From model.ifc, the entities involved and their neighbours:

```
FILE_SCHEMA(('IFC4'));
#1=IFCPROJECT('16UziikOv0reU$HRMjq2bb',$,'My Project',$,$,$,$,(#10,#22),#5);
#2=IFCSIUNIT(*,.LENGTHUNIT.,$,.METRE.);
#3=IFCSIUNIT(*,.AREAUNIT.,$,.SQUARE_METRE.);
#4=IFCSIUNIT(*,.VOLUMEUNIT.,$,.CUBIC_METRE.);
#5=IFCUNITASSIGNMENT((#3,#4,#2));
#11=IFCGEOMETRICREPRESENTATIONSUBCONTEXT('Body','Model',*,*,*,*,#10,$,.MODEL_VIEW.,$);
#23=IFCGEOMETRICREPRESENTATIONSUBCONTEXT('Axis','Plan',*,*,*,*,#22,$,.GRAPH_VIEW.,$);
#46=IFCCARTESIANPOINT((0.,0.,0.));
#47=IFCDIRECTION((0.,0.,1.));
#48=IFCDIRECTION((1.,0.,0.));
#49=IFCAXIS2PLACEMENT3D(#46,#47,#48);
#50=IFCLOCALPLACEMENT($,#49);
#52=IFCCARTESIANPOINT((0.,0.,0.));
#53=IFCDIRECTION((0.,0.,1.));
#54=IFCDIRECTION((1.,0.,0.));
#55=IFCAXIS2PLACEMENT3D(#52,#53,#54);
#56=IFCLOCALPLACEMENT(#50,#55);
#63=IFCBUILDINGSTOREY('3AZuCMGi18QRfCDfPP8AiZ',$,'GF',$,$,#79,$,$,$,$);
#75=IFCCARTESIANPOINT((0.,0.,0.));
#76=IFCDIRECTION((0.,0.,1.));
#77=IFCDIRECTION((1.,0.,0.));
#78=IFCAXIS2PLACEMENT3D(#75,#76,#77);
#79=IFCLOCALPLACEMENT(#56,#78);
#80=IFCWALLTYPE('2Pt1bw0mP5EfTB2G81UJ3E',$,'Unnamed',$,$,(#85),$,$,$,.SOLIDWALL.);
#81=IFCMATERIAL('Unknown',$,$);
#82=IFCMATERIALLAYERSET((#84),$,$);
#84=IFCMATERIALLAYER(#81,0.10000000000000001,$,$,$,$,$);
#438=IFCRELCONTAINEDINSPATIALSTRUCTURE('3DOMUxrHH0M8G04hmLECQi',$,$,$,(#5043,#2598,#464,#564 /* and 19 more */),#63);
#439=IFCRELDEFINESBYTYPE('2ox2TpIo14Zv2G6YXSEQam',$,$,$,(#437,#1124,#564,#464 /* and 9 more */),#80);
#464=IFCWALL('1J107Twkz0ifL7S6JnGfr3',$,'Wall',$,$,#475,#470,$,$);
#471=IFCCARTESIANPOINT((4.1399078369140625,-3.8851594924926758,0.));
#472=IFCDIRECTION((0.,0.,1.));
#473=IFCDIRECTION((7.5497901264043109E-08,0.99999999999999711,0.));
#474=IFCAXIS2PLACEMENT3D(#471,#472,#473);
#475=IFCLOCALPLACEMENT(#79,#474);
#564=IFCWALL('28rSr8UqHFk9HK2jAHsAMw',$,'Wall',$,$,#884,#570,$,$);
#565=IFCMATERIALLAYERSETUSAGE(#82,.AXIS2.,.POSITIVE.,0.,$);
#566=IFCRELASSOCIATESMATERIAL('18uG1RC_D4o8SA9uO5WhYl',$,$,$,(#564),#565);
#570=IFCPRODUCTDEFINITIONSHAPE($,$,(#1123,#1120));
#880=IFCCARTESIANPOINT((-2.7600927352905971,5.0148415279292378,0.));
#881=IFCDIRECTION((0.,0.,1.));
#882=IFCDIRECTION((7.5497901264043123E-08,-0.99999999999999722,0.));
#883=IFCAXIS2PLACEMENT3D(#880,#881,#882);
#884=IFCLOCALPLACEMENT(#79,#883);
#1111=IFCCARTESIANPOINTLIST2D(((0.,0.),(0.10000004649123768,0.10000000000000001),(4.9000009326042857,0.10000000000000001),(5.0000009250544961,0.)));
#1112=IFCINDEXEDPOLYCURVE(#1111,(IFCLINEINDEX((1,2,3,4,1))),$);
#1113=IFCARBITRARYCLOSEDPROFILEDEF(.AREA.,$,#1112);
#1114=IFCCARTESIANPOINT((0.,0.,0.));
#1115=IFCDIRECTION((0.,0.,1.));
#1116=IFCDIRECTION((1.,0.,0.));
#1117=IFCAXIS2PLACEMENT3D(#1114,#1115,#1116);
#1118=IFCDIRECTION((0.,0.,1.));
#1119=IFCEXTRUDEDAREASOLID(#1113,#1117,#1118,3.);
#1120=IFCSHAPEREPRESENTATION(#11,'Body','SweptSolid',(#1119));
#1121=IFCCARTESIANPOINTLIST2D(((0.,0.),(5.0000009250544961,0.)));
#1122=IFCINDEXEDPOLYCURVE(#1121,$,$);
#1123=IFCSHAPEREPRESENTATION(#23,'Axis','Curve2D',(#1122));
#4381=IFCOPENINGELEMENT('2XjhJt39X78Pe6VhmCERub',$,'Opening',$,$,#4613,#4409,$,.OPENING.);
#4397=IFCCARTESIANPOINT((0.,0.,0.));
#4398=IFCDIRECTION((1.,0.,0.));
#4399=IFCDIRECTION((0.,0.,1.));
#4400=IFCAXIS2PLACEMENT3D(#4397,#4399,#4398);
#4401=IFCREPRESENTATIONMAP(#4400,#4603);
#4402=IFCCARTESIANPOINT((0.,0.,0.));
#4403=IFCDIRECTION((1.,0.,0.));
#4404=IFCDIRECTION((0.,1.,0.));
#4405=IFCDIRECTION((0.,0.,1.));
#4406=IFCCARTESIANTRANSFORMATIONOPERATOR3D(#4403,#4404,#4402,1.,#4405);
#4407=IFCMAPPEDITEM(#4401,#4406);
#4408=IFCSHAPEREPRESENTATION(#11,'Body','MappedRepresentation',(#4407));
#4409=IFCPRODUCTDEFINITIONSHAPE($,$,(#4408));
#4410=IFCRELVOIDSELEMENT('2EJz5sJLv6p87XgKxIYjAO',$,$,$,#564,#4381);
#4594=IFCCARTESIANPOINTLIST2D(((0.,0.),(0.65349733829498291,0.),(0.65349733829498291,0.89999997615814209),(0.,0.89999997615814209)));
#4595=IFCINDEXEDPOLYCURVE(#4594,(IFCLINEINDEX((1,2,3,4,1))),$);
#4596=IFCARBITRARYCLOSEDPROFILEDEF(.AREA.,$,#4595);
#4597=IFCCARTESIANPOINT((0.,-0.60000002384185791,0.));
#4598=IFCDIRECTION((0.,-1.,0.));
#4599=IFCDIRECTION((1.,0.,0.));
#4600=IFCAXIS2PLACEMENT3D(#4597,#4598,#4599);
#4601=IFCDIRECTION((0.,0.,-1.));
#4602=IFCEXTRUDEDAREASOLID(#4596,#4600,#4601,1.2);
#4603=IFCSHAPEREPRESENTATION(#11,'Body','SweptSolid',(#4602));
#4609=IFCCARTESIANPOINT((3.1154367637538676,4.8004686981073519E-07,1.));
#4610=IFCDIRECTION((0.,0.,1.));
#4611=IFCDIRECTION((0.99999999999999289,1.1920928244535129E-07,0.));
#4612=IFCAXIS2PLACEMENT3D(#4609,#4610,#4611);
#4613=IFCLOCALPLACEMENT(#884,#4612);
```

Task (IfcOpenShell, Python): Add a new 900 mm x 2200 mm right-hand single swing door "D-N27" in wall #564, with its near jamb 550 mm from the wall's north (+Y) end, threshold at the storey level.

```python
import numpy as np
import ifcopenshell
import ifcopenshell.api.feature
import ifcopenshell.api.geometry
import ifcopenshell.api.root
import ifcopenshell.api.spatial
import ifcopenshell.geom
import ifcopenshell.util.element
import ifcopenshell.util.placement
import ifcopenshell.util.representation
import ifcopenshell.util.shape
import ifcopenshell.util.unit

model = ifcopenshell.open("model.ifc")
unit_scale = ifcopenshell.util.unit.calculate_unit_scale(model)
settings = ifcopenshell.geom.settings()


def volume(element):
    """Net volume in cubic metres, openings subtracted."""
    shape = ifcopenshell.geom.create_shape(settings, element)
    return ifcopenshell.util.shape.get_volume(shape.geometry)


wall = model.by_id(564)
storey = ifcopenshell.util.element.get_container(wall, ifc_class="IfcBuildingStorey")
context = ifcopenshell.util.representation.get_context(model, "Model", "Body", "MODEL_VIEW")
before = volume(wall)

width, height, from_end, sill = 0.9, 2.2, 0.55, 0.0  # metres

# The wall runs along its own X axis, and the end named is its -X end.
wall_shape = ifcopenshell.geom.create_shape(settings, wall)
x, y, z = ifcopenshell.util.shape.get_vertices(wall_shape.geometry).T
start = x.min() + from_end
face, thickness = float(y.min()), float(y.max() - y.min())
wall_matrix = ifcopenshell.util.placement.get_local_placement(wall.ObjectPlacement)
level = ifcopenshell.util.placement.get_local_placement(storey.ObjectPlacement)[2, 3]


def in_wall(x, y):
    """Placement at x, y metres in the wall's axes, at sill height."""
    matrix = wall_matrix.copy()
    matrix[:, 3] = wall_matrix @ np.array([x / unit_scale, y / unit_scale, 0.0, 1.0])
    matrix[2, 3] = level + sill / unit_scale
    return matrix


# Opening: a box that overshoots both wall faces by 50 mm.
opening = ifcopenshell.api.root.create_entity(model, ifc_class="IfcOpeningElement", predefined_type="OPENING")
box = ifcopenshell.api.geometry.add_wall_representation(
    model, context=context, length=width, height=height, thickness=thickness + 0.1
)
ifcopenshell.api.geometry.assign_representation(model, product=opening, representation=box)
ifcopenshell.api.geometry.edit_object_placement(model, product=opening, matrix=in_wall(start, face - 0.05), is_si=False)
ifcopenshell.api.feature.add_feature(model, feature=opening, element=wall)

door = ifcopenshell.api.root.create_entity(model, ifc_class="IfcDoor", name="D-N27", predefined_type="DOOR")
door.OverallWidth, door.OverallHeight = width / unit_scale, height / unit_scale
door.OperationType = "SINGLE_SWING_RIGHT"
body = ifcopenshell.api.geometry.add_door_representation(
    model,
    context=context,
    overall_width=door.OverallWidth,
    overall_height=door.OverallHeight,
    operation_type="SINGLE_SWING_RIGHT",
    lining_properties={"LiningDepth": thickness / unit_scale, "ThresholdDepth": thickness / unit_scale},
)
ifcopenshell.api.geometry.assign_representation(model, product=door, representation=body)
ifcopenshell.api.spatial.assign_container(model, products=[door], relating_structure=storey)
ifcopenshell.api.feature.add_filling(model, opening=opening, element=door)

# The lining spans the wall, so the door starts at the wall face.
ifcopenshell.api.geometry.edit_object_placement(model, product=door, matrix=in_wall(start, face), is_si=False)

after = volume(wall)

print(f"wall volume {before:.3f} -> {after:.3f} m3")

model.write("model_rev.ifc")
```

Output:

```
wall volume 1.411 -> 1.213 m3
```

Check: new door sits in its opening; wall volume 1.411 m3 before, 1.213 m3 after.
